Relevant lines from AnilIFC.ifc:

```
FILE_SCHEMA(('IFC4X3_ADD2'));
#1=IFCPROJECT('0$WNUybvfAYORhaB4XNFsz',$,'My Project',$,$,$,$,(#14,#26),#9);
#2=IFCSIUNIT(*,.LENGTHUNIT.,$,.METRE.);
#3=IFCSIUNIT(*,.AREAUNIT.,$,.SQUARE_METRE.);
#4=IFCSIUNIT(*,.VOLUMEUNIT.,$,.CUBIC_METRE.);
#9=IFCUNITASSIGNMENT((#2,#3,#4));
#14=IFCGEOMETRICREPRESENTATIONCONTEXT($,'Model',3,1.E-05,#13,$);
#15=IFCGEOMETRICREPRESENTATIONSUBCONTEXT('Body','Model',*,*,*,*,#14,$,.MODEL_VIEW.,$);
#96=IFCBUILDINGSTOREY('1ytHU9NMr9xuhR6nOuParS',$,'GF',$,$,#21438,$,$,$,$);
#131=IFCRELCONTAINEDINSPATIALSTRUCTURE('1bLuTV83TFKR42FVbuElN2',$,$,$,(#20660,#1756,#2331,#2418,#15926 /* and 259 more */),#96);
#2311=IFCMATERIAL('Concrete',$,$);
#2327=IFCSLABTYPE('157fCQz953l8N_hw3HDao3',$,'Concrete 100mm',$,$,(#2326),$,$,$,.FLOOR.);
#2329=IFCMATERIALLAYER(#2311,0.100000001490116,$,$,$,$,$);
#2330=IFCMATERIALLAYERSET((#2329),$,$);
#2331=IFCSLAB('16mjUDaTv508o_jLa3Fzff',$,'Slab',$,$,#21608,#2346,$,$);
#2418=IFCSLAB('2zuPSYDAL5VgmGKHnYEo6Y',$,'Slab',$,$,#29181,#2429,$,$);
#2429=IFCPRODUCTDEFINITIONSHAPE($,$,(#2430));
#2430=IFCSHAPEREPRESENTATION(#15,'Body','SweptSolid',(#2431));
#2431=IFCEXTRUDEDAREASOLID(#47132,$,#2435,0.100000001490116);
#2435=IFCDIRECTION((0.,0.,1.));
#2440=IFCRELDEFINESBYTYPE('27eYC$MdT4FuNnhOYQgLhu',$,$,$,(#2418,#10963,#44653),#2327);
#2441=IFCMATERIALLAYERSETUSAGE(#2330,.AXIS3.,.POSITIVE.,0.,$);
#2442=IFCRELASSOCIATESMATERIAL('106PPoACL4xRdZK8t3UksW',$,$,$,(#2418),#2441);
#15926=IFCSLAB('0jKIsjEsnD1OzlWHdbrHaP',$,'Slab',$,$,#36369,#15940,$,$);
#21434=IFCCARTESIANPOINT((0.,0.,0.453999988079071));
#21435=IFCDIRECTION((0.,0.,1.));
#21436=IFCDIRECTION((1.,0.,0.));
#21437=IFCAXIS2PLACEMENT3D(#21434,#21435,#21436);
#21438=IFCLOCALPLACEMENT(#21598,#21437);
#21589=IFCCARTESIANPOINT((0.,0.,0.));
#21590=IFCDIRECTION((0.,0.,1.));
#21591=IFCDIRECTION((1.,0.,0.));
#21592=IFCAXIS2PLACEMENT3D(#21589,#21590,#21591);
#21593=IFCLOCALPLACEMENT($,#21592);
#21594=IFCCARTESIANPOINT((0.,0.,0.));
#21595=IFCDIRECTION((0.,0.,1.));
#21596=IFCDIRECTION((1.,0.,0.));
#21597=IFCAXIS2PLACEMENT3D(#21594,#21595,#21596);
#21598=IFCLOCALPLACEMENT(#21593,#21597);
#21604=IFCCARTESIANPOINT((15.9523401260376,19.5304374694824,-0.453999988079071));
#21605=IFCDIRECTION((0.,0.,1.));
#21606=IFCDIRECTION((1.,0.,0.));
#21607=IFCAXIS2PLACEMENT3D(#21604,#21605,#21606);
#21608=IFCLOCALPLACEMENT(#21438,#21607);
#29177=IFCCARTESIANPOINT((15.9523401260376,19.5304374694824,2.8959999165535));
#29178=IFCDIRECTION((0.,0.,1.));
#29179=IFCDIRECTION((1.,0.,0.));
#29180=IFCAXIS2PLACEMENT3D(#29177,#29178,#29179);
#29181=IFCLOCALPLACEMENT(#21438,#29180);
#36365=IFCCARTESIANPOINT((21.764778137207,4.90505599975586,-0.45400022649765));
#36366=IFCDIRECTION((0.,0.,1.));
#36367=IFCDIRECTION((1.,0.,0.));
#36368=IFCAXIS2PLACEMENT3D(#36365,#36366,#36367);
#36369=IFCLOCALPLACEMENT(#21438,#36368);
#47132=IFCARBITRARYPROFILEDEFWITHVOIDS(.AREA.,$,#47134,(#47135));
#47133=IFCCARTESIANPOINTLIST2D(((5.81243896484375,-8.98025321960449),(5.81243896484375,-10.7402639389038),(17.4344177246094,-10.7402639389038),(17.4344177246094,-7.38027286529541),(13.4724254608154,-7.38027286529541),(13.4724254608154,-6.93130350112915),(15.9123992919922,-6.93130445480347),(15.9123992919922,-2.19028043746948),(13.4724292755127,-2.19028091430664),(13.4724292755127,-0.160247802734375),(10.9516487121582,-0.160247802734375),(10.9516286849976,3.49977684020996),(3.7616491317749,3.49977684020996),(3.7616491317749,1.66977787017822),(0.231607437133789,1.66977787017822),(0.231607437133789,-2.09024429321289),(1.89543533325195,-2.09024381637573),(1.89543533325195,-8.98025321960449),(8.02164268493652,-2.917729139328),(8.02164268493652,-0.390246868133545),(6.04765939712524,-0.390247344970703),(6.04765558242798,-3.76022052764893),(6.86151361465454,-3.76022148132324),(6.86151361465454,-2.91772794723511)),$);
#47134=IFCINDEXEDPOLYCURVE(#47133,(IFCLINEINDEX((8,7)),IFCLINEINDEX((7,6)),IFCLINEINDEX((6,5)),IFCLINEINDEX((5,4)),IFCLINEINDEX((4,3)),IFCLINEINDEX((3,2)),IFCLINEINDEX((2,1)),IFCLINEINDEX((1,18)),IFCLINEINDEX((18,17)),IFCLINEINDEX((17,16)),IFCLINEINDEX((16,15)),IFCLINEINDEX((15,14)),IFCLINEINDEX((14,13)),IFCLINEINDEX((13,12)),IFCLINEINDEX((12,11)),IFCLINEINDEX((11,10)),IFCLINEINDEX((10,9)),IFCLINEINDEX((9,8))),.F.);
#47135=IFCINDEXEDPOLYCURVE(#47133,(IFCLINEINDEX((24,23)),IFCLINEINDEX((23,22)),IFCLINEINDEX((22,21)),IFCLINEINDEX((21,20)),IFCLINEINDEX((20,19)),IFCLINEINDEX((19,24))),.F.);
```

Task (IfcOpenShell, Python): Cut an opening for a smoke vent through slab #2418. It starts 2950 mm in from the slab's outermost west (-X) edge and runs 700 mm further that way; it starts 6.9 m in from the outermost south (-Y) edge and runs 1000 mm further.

```python
import numpy as np
import ifcopenshell
import ifcopenshell.api.feature
import ifcopenshell.api.geometry
import ifcopenshell.api.root
import ifcopenshell.geom
import ifcopenshell.util.placement
import ifcopenshell.util.representation
import ifcopenshell.util.shape
import ifcopenshell.util.unit

model = ifcopenshell.open("AnilIFC.ifc")
unit_scale = ifcopenshell.util.unit.calculate_unit_scale(model)
settings = ifcopenshell.geom.settings()


def volume(element):
    """Net volume in cubic metres, openings subtracted."""
    shape = ifcopenshell.geom.create_shape(settings, element)
    return ifcopenshell.util.shape.get_volume(shape.geometry)


slab = model.by_guid("2zuPSYDAL5VgmGKHnYEo6Y")
before = volume(slab)

# Extent in the slab's own axes, in metres. The edges named are its -X and -Y sides.
slab_shape = ifcopenshell.geom.create_shape(settings, slab)
vertices = ifcopenshell.util.shape.get_vertices(slab_shape.geometry)
x_min, y_min, bottom = vertices.min(axis=0)
top = vertices[:, 2].max()

opening = ifcopenshell.api.root.create_entity(model, ifc_class="IfcOpeningElement", name="Smoke vent opening", predefined_type="OPENING")
context = ifcopenshell.util.representation.get_context(model, "Model", "Body", "MODEL_VIEW")
width, depth = 0.7, 1
outline = [(0.0, 0.0), (width, 0.0), (width, depth), (0.0, depth), (0.0, 0.0)]
# Overshoot both faces by 50 mm so the cut is clean.
shape = ifcopenshell.api.geometry.add_slab_representation(
    model, context=context, depth=top - bottom + 0.1, polyline=outline
)
ifcopenshell.api.geometry.assign_representation(model, product=opening, representation=shape)

matrix = ifcopenshell.util.placement.get_local_placement(slab.ObjectPlacement)
matrix[:, 3] = matrix @ np.append(np.array([x_min + 2.95, y_min + 6.9, bottom - 0.05]) / unit_scale, 1.0)
ifcopenshell.api.geometry.edit_object_placement(model, product=opening, matrix=matrix, is_si=False)
ifcopenshell.api.feature.add_feature(model, feature=opening, element=slab)

after = volume(slab)

print(f"slab volume {before:.3f} -> {after:.3f} m3")

model.write("AnilIFC_updated.ifc")
```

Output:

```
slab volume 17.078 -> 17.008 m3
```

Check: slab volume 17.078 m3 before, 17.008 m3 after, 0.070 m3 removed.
